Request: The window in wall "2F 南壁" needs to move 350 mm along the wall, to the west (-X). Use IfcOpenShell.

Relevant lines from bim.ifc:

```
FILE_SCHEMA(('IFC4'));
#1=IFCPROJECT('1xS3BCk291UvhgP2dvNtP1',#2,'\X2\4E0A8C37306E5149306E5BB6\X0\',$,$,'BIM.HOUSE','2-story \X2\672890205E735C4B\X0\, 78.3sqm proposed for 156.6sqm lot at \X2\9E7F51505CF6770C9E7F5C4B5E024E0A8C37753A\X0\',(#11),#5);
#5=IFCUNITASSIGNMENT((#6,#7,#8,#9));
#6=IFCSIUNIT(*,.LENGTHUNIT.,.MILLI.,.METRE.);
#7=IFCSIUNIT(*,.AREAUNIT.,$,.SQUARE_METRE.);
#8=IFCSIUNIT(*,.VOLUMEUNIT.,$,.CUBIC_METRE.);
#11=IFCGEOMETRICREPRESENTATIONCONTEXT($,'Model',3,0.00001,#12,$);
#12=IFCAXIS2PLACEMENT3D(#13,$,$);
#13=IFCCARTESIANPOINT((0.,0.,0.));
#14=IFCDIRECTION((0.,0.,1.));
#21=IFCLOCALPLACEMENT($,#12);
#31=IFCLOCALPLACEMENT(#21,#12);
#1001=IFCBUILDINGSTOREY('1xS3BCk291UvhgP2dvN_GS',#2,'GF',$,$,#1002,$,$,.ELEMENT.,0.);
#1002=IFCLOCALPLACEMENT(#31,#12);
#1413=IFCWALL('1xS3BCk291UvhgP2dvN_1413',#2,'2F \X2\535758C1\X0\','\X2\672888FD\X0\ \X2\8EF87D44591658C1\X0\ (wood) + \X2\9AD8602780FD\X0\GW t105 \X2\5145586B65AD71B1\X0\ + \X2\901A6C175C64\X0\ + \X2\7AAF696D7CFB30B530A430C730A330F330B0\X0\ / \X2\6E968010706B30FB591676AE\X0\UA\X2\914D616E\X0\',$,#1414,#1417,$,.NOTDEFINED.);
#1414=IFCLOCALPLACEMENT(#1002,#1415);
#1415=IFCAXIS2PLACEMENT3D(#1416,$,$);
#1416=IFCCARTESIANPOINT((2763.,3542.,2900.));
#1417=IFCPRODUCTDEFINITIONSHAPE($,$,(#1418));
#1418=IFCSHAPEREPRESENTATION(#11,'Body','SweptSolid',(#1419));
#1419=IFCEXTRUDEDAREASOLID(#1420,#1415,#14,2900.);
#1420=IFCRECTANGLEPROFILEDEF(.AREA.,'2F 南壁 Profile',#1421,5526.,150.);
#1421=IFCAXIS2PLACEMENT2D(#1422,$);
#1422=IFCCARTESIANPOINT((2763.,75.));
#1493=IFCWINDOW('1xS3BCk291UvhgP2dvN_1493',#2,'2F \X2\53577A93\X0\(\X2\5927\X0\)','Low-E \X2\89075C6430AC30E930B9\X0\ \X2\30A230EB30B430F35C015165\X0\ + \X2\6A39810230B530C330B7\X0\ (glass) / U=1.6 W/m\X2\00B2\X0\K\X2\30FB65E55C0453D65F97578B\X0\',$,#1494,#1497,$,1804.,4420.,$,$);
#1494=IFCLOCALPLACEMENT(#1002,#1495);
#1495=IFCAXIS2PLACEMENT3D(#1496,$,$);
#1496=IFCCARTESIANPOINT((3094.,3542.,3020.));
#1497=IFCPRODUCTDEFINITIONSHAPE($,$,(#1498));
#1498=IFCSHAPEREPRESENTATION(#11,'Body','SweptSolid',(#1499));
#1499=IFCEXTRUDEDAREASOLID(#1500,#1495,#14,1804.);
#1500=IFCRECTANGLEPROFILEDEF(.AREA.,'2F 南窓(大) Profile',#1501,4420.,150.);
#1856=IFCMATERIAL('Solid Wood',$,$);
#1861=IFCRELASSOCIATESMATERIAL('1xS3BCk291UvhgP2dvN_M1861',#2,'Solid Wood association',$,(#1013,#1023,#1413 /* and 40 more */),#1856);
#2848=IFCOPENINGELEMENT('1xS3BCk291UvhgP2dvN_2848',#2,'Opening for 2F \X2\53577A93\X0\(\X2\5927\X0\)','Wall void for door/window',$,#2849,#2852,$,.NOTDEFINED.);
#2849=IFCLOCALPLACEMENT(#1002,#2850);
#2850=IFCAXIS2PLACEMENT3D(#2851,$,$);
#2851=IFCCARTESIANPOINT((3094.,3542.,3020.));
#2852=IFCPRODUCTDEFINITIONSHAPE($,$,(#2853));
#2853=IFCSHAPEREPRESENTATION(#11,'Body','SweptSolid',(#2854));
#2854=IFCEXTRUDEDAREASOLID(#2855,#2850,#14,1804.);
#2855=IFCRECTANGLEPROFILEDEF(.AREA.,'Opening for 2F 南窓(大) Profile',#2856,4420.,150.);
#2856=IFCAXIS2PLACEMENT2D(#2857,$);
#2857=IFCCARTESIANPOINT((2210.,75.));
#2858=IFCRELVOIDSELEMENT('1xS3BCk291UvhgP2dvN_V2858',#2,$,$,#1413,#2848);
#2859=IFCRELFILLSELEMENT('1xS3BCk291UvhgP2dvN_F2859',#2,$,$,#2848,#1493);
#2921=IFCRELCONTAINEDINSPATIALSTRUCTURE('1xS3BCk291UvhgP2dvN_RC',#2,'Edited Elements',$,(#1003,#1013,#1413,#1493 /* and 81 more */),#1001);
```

```python
import ifcopenshell
import ifcopenshell.api.geometry
import ifcopenshell.util.placement
import ifcopenshell.util.unit

model = ifcopenshell.open("bim.ifc")
unit_scale = ifcopenshell.util.unit.calculate_unit_scale(model)

window = model.by_guid("1xS3BCk291UvhgP2dvN_1493")
opening = window.FillsVoids[0].RelatingOpeningElement
wall = opening.VoidsElements[0].RelatingBuildingElement

wall_matrix = ifcopenshell.util.placement.get_local_placement(wall.ObjectPlacement)
shift = wall_matrix[:3, 0] * -0.35 / unit_scale
before = ifcopenshell.util.placement.get_local_placement(window.ObjectPlacement)[:3, 3].copy()

# The window is not placed relative to its opening, so move both.
for product in (opening, window):
    matrix = ifcopenshell.util.placement.get_local_placement(product.ObjectPlacement)
    matrix[:3, 3] += shift
    ifcopenshell.api.geometry.edit_object_placement(model, product=product, matrix=matrix, is_si=False)

after = ifcopenshell.util.placement.get_local_placement(window.ObjectPlacement)[:3, 3]
print("window moved by", (after - before).round(3) + 0.0)

model.write("bim_updated.ifc")
```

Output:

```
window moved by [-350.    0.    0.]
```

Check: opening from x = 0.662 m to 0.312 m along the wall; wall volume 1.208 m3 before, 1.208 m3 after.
